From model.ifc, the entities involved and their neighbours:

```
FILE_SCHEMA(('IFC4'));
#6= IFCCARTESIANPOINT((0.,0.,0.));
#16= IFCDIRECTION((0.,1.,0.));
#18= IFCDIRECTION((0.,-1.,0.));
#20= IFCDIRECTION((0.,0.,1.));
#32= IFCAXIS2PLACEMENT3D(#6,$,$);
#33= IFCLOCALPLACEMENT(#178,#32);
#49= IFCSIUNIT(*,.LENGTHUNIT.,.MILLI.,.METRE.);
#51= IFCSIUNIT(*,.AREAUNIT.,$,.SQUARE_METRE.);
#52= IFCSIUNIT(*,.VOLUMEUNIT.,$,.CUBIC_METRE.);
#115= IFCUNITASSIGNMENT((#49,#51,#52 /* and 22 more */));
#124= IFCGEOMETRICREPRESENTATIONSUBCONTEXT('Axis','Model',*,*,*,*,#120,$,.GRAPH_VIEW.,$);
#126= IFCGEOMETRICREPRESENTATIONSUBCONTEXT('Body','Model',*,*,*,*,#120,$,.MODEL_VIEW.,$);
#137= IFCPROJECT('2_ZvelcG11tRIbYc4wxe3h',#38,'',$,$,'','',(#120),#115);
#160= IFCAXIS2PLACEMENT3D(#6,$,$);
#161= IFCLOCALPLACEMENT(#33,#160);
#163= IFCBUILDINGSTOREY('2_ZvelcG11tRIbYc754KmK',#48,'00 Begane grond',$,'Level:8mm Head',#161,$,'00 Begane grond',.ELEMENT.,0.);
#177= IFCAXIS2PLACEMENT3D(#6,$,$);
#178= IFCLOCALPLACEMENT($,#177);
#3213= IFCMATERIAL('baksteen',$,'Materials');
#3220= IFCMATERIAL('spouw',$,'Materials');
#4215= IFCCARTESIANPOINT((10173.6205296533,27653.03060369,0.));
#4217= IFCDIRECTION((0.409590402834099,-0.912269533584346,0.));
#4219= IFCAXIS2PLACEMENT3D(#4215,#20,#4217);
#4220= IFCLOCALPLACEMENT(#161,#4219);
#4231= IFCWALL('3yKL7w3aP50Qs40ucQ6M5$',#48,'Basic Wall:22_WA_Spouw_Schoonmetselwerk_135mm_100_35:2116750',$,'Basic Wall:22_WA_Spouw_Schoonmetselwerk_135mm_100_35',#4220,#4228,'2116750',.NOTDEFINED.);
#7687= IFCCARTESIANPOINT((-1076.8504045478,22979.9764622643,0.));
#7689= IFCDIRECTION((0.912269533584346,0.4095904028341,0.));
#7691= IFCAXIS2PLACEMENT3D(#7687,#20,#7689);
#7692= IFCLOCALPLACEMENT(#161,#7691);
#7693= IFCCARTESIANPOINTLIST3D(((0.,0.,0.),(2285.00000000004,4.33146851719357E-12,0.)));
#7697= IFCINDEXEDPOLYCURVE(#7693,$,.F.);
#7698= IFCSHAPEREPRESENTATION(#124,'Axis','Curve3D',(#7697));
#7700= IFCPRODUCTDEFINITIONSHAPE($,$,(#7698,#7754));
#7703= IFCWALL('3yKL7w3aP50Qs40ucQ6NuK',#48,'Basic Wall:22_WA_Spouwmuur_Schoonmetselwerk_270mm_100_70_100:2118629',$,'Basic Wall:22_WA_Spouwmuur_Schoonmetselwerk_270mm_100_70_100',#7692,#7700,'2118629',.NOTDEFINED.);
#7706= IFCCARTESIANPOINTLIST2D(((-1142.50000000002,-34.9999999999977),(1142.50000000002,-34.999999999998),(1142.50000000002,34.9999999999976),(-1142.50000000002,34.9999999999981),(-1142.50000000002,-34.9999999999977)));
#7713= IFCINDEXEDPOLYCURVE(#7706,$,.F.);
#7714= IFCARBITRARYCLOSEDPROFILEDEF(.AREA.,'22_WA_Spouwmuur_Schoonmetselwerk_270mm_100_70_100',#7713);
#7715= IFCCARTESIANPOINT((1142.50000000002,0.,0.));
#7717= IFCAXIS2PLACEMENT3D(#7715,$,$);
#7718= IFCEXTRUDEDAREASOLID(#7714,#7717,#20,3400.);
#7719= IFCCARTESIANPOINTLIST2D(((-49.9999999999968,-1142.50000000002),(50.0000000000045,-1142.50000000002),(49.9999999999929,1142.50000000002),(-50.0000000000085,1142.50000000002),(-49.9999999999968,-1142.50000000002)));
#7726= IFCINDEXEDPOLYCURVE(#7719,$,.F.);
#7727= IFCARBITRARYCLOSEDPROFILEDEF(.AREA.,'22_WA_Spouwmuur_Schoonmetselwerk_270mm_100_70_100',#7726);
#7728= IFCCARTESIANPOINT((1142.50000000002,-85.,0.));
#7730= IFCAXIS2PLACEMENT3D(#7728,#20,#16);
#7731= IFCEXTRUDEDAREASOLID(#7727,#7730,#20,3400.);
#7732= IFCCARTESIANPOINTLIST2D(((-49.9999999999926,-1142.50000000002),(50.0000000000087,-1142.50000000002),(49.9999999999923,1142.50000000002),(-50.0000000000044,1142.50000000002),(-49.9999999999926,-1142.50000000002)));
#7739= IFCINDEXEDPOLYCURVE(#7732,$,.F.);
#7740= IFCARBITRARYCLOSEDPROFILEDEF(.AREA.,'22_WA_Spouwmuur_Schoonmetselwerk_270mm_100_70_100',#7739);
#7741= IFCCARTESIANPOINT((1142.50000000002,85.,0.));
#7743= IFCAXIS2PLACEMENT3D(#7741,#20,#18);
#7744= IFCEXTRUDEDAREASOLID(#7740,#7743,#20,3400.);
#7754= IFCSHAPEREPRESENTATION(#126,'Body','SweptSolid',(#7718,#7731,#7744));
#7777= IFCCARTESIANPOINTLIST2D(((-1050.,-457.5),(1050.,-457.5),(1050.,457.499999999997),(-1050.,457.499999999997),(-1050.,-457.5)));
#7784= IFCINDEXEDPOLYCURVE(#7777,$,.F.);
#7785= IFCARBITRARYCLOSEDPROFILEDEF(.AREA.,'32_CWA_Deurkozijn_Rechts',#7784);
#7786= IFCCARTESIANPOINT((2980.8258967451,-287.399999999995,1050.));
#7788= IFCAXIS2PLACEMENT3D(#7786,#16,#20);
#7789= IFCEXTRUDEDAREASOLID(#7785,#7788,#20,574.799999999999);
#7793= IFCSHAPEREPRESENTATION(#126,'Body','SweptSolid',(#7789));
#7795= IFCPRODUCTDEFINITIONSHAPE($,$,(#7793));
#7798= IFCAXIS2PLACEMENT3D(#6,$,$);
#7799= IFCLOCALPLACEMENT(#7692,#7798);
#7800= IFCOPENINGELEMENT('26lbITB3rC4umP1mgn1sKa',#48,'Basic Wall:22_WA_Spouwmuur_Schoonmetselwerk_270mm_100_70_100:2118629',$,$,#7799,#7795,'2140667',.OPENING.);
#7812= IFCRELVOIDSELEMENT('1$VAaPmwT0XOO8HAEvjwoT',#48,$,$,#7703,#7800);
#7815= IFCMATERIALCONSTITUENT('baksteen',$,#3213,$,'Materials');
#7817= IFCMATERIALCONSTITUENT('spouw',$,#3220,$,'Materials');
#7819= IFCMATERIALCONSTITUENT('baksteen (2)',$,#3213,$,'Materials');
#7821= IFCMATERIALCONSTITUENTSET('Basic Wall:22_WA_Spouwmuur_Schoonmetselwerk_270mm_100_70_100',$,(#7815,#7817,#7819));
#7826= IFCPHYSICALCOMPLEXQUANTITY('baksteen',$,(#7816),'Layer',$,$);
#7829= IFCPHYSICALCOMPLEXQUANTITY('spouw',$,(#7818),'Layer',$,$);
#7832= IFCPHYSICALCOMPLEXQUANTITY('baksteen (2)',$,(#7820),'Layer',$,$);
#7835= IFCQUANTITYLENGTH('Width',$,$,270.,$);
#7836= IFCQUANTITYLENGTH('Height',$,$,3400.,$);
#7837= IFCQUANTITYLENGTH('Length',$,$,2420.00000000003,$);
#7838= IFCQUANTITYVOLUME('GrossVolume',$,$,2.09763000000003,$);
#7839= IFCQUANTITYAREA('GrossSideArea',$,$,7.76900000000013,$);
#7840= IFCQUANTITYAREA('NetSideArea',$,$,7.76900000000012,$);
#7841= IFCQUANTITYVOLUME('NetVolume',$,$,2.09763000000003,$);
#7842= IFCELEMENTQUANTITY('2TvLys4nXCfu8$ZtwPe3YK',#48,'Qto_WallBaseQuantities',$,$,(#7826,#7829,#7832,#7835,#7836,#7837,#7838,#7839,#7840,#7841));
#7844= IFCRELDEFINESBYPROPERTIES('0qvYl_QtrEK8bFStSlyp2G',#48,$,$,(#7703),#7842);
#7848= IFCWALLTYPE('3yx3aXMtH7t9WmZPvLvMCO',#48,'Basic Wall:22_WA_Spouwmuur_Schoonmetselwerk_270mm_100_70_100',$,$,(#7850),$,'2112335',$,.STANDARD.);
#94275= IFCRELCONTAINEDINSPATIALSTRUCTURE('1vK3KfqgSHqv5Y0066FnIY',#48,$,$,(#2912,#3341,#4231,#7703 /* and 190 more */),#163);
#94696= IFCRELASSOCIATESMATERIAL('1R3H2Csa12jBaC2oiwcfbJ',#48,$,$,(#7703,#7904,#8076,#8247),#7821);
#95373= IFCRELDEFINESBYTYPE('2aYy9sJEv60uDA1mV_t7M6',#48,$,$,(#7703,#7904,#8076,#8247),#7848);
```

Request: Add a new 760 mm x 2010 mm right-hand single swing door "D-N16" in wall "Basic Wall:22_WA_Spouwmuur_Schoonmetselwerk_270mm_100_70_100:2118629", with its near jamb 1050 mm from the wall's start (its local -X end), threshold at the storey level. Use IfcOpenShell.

```python
import numpy as np
import ifcopenshell
import ifcopenshell.api.feature
import ifcopenshell.api.geometry
import ifcopenshell.api.pset
import ifcopenshell.api.root
import ifcopenshell.api.spatial
import ifcopenshell.geom
import ifcopenshell.util.element
import ifcopenshell.util.placement
import ifcopenshell.util.representation
import ifcopenshell.util.shape
import ifcopenshell.util.unit

model = ifcopenshell.open("model.ifc")
unit_scale = ifcopenshell.util.unit.calculate_unit_scale(model)
area_scale = ifcopenshell.util.unit.calculate_unit_scale(model, "AREAUNIT")
volume_scale = ifcopenshell.util.unit.calculate_unit_scale(model, "VOLUMEUNIT")
settings = ifcopenshell.geom.settings()


def volume(element):
    """Net volume in cubic metres, openings subtracted."""
    shape = ifcopenshell.geom.create_shape(settings, element)
    return ifcopenshell.util.shape.get_volume(shape.geometry)


wall = model.by_guid("3yKL7w3aP50Qs40ucQ6NuK")
storey = ifcopenshell.util.element.get_container(wall, ifc_class="IfcBuildingStorey")
context = ifcopenshell.util.representation.get_context(model, "Model", "Body", "MODEL_VIEW")
before = volume(wall)

width, height, from_end, sill = 0.76, 2.01, 1.05, 0.0  # metres

# The wall runs along its own X axis, and the end named is its -X end.
wall_shape = ifcopenshell.geom.create_shape(settings, wall)
x, y, z = ifcopenshell.util.shape.get_vertices(wall_shape.geometry).T
start = x.min() + from_end
face, thickness = float(y.min()), float(y.max() - y.min())
wall_matrix = ifcopenshell.util.placement.get_local_placement(wall.ObjectPlacement)
level = ifcopenshell.util.placement.get_local_placement(storey.ObjectPlacement)[2, 3]


def in_wall(x, y):
    """Placement at x, y metres in the wall's axes, at sill height."""
    matrix = wall_matrix.copy()
    matrix[:, 3] = wall_matrix @ np.array([x / unit_scale, y / unit_scale, 0.0, 1.0])
    matrix[2, 3] = level + sill / unit_scale
    return matrix


# Opening: a box that overshoots both wall faces by 50 mm.
opening = ifcopenshell.api.root.create_entity(model, ifc_class="IfcOpeningElement", predefined_type="OPENING")
box = ifcopenshell.api.geometry.add_wall_representation(
    model, context=context, length=width, height=height, thickness=thickness + 0.1
)
ifcopenshell.api.geometry.assign_representation(model, product=opening, representation=box)
ifcopenshell.api.geometry.edit_object_placement(model, product=opening, matrix=in_wall(start, face - 0.05), is_si=False)
ifcopenshell.api.feature.add_feature(model, feature=opening, element=wall)

door = ifcopenshell.api.root.create_entity(model, ifc_class="IfcDoor", name="D-N16", predefined_type="DOOR")
door.OverallWidth, door.OverallHeight = width / unit_scale, height / unit_scale
door.OperationType = "SINGLE_SWING_RIGHT"
body = ifcopenshell.api.geometry.add_door_representation(
    model,
    context=context,
    overall_width=door.OverallWidth,
    overall_height=door.OverallHeight,
    operation_type="SINGLE_SWING_RIGHT",
    lining_properties={"LiningDepth": thickness / unit_scale, "ThresholdDepth": thickness / unit_scale},
)
ifcopenshell.api.geometry.assign_representation(model, product=door, representation=body)
ifcopenshell.api.spatial.assign_container(model, products=[door], relating_structure=storey)
ifcopenshell.api.feature.add_filling(model, opening=opening, element=door)

# The lining spans the wall, so the door starts at the wall face.
ifcopenshell.api.geometry.edit_object_placement(model, product=door, matrix=in_wall(start, face), is_si=False)

after = volume(wall)

# Update the wall's stored quantities.
qto = model.by_id(ifcopenshell.util.element.get_pset(wall, "Qto_WallBaseQuantities", should_inherit=False)["id"])
ifcopenshell.api.pset.edit_qto(model, qto=qto, properties={
    "NetSideArea": after / thickness / area_scale,
    "NetVolume": after / volume_scale,
})

print(f"wall volume {before:.3f} -> {after:.3f} m3")

model.write("model_rev.ifc")
```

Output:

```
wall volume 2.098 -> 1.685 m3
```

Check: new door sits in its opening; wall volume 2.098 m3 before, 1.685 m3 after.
